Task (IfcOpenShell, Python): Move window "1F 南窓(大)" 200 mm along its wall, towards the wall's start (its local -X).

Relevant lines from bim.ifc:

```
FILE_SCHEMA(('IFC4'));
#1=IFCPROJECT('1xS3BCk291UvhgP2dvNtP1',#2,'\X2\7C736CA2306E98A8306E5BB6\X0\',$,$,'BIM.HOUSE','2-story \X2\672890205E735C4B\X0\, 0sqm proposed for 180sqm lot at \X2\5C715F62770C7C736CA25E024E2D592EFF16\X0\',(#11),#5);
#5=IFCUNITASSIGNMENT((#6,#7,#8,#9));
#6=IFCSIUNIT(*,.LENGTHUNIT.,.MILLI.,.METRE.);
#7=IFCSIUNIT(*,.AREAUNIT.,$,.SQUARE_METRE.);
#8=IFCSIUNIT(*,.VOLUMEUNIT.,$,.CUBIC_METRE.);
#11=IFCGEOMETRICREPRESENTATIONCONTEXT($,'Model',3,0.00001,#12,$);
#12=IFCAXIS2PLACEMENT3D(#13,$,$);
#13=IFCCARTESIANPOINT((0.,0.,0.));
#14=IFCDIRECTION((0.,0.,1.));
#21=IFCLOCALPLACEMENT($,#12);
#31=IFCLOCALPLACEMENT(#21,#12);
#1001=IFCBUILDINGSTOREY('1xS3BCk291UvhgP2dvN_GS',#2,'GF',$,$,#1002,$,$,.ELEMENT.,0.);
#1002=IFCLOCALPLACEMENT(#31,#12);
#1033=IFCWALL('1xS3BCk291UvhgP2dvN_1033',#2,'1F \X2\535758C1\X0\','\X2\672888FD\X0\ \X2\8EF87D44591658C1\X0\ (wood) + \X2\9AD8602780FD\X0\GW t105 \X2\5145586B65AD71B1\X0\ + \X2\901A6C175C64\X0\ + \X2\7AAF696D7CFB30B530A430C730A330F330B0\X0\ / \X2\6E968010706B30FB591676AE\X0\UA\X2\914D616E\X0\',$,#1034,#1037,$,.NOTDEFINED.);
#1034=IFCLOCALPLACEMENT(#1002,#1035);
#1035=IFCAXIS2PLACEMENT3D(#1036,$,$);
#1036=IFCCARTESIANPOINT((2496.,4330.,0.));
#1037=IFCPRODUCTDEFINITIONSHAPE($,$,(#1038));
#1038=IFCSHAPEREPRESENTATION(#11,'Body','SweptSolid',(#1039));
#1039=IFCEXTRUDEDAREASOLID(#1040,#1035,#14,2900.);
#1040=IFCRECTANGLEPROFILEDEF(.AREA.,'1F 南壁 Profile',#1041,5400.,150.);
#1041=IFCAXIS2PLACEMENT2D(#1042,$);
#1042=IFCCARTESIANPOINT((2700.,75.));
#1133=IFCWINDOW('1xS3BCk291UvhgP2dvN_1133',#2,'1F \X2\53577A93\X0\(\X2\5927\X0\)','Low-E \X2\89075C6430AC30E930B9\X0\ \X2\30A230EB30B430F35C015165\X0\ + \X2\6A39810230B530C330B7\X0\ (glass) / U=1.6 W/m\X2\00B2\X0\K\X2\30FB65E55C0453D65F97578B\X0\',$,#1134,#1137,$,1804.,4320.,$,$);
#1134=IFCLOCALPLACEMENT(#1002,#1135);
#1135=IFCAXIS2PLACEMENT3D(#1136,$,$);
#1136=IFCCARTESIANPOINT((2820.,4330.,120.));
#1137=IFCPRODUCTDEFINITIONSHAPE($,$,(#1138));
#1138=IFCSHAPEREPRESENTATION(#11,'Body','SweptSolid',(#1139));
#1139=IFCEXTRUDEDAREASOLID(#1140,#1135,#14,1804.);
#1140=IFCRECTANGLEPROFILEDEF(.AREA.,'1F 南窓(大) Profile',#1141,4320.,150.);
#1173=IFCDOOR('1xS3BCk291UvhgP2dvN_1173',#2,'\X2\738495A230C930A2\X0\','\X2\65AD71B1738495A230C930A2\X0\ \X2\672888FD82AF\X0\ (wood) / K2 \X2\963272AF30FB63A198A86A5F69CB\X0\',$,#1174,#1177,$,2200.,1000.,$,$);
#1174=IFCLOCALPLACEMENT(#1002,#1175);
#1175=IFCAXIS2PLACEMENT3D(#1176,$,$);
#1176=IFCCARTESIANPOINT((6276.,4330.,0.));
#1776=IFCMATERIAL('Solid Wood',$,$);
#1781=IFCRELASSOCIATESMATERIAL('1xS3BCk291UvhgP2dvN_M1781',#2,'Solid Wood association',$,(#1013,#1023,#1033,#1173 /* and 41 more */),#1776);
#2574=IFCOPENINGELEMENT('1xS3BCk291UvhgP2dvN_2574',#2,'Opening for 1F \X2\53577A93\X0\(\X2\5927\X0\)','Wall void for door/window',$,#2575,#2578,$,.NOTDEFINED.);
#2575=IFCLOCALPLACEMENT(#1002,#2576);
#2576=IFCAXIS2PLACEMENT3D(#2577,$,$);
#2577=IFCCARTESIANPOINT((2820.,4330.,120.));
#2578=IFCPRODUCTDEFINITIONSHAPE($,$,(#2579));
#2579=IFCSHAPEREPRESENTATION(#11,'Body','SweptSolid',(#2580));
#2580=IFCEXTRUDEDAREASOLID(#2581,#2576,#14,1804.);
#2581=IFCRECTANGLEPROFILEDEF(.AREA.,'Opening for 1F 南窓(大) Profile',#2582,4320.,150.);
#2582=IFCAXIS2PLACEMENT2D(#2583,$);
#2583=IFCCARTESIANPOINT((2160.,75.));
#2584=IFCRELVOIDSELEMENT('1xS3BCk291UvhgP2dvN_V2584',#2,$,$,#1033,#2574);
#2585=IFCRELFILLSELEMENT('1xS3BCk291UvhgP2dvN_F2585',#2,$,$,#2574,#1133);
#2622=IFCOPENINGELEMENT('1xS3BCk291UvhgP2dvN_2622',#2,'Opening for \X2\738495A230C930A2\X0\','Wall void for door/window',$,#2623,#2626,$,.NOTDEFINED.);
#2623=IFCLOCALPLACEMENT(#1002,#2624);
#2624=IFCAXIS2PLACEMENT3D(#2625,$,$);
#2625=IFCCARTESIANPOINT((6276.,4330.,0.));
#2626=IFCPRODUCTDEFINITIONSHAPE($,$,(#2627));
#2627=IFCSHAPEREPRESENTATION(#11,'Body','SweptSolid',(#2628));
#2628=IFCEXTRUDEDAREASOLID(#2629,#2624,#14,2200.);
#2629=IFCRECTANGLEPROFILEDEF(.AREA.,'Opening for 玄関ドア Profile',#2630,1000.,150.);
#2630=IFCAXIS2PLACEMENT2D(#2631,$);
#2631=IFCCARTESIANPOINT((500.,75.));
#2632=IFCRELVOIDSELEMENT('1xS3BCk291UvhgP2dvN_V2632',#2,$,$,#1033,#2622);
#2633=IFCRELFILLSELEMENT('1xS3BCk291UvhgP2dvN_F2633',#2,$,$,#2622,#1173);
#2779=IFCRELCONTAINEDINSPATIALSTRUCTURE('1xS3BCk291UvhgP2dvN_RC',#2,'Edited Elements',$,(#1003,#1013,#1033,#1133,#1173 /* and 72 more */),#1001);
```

```python
import ifcopenshell
import ifcopenshell.api.geometry
import ifcopenshell.util.placement
import ifcopenshell.util.unit

model = ifcopenshell.open("bim.ifc")
unit_scale = ifcopenshell.util.unit.calculate_unit_scale(model)

window = model.by_id(1133)
opening = window.FillsVoids[0].RelatingOpeningElement
wall = opening.VoidsElements[0].RelatingBuildingElement

wall_matrix = ifcopenshell.util.placement.get_local_placement(wall.ObjectPlacement)
shift = wall_matrix[:3, 0] * -0.2 / unit_scale
before = ifcopenshell.util.placement.get_local_placement(window.ObjectPlacement)[:3, 3].copy()

# The window is not placed relative to its opening, so move both.
for product in (opening, window):
    matrix = ifcopenshell.util.placement.get_local_placement(product.ObjectPlacement)
    matrix[:3, 3] += shift
    ifcopenshell.api.geometry.edit_object_placement(model, product=product, matrix=matrix, is_si=False)

after = ifcopenshell.util.placement.get_local_placement(window.ObjectPlacement)[:3, 3]
print("window moved by", (after - before).round(3) + 0.0)

model.write("bim_updated.ifc")
```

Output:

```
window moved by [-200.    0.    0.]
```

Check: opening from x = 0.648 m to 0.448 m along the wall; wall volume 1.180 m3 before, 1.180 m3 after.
